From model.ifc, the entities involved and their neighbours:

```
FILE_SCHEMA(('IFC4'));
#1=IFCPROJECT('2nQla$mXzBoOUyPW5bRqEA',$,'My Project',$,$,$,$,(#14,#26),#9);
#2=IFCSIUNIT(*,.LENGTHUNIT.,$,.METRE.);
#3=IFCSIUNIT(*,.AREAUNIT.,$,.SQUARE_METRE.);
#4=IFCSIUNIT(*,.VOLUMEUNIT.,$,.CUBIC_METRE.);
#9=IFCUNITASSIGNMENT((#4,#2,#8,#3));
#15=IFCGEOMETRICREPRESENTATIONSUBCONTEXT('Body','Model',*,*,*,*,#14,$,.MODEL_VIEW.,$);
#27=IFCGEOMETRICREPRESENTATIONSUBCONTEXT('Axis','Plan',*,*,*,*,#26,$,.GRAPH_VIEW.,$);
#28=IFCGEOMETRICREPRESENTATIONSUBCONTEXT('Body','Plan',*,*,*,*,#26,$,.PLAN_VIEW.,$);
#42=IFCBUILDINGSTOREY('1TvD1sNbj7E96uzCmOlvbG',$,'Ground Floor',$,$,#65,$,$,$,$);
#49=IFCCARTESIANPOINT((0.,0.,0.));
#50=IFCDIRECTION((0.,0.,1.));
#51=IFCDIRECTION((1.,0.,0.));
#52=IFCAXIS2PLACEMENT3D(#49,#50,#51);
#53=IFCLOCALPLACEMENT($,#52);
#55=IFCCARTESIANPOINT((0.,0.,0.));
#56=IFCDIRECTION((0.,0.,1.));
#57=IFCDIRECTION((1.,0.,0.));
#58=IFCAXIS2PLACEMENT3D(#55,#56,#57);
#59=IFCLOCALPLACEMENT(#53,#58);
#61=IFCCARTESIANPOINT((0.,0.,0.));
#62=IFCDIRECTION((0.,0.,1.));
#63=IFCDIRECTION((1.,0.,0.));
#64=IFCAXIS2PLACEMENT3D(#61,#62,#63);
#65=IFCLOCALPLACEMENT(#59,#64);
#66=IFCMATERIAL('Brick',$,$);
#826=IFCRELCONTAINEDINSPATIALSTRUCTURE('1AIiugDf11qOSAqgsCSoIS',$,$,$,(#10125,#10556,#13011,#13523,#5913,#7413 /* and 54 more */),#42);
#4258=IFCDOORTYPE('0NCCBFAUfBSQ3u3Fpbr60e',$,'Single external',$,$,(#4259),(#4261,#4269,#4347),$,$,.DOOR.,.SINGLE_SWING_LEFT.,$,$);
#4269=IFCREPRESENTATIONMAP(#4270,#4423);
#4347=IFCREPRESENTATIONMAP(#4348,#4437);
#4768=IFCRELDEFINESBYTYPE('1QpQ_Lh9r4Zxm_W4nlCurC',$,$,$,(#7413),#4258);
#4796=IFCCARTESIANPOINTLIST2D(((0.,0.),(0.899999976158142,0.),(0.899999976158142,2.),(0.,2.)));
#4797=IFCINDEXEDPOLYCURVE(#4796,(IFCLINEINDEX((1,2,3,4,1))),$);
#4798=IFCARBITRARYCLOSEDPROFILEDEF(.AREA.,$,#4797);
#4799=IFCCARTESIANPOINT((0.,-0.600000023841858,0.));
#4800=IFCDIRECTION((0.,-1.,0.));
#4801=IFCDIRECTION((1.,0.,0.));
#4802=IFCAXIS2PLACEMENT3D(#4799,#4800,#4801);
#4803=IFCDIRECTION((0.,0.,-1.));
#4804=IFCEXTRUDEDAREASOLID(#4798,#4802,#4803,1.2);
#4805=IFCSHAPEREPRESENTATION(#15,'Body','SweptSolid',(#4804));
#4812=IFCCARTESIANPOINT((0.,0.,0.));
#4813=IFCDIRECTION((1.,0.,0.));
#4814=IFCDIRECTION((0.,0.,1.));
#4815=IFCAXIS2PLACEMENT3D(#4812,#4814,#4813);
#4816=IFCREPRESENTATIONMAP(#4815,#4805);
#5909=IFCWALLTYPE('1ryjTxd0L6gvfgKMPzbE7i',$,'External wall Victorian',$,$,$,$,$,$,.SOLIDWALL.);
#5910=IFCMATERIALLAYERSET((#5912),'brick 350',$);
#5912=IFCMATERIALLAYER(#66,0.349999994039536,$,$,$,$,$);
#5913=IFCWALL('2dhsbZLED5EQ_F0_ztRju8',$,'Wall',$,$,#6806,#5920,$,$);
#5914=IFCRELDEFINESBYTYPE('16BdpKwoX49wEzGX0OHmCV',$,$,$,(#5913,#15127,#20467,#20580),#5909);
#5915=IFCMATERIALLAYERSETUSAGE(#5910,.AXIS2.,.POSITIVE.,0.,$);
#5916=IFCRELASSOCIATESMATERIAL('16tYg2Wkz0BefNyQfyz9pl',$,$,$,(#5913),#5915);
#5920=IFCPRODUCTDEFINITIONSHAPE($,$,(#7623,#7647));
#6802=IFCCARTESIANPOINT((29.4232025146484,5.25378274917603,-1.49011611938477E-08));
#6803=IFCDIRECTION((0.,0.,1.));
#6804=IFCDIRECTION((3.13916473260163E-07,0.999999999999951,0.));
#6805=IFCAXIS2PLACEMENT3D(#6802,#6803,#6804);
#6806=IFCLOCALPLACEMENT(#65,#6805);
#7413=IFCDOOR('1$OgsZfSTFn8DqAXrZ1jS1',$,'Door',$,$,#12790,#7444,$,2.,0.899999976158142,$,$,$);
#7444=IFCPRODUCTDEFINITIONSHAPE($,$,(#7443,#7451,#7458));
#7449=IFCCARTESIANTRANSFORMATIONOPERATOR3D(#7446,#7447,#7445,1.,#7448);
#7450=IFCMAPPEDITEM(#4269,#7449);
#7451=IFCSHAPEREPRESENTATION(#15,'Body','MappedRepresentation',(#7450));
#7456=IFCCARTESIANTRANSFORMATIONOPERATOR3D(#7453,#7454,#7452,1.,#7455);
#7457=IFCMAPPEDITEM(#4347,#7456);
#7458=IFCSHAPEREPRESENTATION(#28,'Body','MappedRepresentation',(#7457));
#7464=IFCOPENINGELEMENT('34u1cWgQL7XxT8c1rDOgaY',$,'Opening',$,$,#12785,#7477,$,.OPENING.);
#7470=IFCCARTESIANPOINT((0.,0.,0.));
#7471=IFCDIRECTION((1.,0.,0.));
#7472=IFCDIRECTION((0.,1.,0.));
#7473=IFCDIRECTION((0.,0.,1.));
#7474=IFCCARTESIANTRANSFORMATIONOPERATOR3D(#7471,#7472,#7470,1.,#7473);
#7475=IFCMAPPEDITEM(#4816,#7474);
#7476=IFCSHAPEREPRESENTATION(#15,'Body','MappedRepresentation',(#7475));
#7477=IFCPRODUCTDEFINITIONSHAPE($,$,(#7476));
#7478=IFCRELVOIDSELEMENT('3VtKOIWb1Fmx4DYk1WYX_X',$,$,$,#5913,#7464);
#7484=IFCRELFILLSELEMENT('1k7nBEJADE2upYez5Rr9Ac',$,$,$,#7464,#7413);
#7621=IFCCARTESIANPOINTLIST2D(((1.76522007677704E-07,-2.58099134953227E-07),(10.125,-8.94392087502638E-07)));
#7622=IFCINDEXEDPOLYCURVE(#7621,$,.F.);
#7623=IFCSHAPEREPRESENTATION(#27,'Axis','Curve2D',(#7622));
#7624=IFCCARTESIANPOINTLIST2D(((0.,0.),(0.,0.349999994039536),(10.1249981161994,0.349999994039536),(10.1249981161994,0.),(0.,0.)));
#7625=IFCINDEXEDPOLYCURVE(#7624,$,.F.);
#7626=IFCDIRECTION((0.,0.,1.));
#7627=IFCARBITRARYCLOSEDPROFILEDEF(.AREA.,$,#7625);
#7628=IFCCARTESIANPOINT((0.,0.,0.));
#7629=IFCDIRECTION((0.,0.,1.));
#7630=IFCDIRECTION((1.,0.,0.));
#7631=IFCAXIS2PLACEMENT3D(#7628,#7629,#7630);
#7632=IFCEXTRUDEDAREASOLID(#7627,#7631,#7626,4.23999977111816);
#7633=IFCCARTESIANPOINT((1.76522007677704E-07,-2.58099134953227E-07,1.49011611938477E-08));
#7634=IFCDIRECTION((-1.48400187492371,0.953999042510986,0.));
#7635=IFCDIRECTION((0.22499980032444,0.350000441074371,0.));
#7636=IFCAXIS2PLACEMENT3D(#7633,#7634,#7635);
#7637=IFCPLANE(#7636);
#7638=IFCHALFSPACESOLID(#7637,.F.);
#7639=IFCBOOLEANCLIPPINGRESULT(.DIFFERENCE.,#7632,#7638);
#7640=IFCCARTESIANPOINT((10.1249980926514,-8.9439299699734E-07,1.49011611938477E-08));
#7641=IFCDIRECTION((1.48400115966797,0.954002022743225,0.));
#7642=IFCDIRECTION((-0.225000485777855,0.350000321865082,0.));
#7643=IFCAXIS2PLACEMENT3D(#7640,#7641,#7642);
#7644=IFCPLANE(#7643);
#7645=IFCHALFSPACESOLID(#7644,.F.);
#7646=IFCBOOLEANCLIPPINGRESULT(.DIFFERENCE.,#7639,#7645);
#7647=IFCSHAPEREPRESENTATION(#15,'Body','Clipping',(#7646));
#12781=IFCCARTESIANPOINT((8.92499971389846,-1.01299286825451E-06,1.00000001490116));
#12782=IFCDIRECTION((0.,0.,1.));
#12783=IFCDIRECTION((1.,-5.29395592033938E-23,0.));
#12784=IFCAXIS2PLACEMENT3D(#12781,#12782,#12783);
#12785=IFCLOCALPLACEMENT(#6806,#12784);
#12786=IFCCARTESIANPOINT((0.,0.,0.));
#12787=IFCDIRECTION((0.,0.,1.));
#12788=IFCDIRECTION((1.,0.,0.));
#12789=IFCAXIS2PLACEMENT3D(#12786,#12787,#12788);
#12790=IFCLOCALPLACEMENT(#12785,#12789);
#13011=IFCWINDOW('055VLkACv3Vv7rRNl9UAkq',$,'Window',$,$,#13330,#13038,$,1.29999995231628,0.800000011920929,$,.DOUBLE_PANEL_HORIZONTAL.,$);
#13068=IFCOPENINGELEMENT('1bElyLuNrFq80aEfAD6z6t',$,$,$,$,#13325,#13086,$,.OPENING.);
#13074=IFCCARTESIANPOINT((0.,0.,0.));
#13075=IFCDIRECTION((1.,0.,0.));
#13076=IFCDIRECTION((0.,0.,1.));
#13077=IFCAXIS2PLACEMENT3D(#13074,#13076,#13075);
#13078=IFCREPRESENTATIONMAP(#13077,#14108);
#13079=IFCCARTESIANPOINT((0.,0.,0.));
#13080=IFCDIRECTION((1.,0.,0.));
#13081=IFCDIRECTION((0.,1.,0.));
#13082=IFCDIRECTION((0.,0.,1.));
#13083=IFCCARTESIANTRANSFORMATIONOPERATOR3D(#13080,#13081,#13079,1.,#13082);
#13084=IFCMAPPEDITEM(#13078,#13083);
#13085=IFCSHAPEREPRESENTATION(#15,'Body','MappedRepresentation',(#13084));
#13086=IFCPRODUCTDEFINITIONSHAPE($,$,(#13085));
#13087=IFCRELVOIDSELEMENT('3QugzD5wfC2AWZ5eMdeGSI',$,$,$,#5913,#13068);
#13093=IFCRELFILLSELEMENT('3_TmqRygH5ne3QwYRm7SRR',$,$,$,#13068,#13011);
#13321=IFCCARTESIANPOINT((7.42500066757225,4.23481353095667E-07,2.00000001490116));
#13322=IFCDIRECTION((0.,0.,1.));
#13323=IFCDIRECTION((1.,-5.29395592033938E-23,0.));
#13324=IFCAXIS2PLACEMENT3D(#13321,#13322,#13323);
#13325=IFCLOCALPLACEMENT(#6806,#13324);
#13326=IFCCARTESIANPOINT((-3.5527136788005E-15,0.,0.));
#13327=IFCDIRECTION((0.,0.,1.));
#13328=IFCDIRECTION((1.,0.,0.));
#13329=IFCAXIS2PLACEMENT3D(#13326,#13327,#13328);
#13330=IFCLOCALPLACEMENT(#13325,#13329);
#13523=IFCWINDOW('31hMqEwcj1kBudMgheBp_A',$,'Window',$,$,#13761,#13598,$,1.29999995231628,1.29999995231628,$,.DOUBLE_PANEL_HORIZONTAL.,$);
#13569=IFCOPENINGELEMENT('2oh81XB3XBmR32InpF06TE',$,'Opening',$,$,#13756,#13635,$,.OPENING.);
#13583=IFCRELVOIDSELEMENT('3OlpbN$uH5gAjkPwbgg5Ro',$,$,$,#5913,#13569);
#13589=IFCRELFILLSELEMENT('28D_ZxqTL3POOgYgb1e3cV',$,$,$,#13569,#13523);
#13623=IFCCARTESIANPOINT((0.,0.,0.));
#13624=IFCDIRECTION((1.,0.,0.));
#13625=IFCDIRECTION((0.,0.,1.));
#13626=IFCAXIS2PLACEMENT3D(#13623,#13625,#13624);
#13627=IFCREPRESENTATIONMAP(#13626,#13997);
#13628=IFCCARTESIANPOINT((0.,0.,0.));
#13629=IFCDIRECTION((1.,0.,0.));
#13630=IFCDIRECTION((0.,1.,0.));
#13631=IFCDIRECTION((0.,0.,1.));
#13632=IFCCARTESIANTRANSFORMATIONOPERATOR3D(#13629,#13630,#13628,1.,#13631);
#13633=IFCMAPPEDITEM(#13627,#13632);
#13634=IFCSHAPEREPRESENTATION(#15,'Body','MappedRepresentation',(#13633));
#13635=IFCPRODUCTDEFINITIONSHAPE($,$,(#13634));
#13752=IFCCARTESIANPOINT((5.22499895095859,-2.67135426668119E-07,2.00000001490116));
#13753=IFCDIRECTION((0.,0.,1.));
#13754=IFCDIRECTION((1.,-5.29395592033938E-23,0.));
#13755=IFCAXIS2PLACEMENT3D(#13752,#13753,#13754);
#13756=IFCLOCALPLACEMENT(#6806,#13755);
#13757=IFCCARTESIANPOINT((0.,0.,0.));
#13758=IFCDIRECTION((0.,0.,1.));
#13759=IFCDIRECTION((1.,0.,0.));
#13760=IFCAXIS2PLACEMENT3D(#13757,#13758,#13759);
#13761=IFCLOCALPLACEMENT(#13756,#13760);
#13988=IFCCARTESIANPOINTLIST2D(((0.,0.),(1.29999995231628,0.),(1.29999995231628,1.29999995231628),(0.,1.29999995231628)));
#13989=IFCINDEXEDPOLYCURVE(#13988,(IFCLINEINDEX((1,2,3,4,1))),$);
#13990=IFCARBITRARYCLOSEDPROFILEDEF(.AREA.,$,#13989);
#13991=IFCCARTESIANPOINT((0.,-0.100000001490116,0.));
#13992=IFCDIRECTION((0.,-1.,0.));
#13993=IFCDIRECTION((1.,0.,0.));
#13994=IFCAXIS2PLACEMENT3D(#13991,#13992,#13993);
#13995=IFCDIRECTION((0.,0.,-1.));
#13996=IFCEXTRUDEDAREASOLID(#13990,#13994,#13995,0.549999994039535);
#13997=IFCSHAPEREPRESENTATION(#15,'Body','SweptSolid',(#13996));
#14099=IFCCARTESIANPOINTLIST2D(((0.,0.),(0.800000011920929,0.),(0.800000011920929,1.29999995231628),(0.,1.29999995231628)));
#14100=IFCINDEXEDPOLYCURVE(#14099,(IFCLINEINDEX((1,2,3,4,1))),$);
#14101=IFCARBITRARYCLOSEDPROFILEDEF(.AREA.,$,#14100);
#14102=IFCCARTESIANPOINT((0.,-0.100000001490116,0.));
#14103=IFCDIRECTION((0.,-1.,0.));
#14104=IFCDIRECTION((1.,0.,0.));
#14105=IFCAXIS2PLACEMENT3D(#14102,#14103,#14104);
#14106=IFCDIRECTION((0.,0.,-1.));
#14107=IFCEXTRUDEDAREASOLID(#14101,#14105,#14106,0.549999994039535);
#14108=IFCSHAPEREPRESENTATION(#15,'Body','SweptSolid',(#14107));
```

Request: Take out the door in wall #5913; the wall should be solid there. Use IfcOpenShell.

```python
import ifcopenshell
import ifcopenshell.api.feature
import ifcopenshell.api.root
import ifcopenshell.geom
import ifcopenshell.util.shape

model = ifcopenshell.open("model.ifc")
settings = ifcopenshell.geom.settings()


def volume(element):
    """Net volume in cubic metres, openings subtracted."""
    shape = ifcopenshell.geom.create_shape(settings, element)
    return ifcopenshell.util.shape.get_volume(shape.geometry)


door = model.by_guid("1$OgsZfSTFn8DqAXrZ1jS1")
opening = door.FillsVoids[0].RelatingOpeningElement
wall = opening.VoidsElements[0].RelatingBuildingElement
before = volume(wall)

ifcopenshell.api.root.remove_product(model, product=door)
ifcopenshell.api.feature.remove_feature(model, feature=opening)

after = volume(wall)

print(f"wall volume {before:.3f} -> {after:.3f} m3")

model.write("model_edited.ifc")
```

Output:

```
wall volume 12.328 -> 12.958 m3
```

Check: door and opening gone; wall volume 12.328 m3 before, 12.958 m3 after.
